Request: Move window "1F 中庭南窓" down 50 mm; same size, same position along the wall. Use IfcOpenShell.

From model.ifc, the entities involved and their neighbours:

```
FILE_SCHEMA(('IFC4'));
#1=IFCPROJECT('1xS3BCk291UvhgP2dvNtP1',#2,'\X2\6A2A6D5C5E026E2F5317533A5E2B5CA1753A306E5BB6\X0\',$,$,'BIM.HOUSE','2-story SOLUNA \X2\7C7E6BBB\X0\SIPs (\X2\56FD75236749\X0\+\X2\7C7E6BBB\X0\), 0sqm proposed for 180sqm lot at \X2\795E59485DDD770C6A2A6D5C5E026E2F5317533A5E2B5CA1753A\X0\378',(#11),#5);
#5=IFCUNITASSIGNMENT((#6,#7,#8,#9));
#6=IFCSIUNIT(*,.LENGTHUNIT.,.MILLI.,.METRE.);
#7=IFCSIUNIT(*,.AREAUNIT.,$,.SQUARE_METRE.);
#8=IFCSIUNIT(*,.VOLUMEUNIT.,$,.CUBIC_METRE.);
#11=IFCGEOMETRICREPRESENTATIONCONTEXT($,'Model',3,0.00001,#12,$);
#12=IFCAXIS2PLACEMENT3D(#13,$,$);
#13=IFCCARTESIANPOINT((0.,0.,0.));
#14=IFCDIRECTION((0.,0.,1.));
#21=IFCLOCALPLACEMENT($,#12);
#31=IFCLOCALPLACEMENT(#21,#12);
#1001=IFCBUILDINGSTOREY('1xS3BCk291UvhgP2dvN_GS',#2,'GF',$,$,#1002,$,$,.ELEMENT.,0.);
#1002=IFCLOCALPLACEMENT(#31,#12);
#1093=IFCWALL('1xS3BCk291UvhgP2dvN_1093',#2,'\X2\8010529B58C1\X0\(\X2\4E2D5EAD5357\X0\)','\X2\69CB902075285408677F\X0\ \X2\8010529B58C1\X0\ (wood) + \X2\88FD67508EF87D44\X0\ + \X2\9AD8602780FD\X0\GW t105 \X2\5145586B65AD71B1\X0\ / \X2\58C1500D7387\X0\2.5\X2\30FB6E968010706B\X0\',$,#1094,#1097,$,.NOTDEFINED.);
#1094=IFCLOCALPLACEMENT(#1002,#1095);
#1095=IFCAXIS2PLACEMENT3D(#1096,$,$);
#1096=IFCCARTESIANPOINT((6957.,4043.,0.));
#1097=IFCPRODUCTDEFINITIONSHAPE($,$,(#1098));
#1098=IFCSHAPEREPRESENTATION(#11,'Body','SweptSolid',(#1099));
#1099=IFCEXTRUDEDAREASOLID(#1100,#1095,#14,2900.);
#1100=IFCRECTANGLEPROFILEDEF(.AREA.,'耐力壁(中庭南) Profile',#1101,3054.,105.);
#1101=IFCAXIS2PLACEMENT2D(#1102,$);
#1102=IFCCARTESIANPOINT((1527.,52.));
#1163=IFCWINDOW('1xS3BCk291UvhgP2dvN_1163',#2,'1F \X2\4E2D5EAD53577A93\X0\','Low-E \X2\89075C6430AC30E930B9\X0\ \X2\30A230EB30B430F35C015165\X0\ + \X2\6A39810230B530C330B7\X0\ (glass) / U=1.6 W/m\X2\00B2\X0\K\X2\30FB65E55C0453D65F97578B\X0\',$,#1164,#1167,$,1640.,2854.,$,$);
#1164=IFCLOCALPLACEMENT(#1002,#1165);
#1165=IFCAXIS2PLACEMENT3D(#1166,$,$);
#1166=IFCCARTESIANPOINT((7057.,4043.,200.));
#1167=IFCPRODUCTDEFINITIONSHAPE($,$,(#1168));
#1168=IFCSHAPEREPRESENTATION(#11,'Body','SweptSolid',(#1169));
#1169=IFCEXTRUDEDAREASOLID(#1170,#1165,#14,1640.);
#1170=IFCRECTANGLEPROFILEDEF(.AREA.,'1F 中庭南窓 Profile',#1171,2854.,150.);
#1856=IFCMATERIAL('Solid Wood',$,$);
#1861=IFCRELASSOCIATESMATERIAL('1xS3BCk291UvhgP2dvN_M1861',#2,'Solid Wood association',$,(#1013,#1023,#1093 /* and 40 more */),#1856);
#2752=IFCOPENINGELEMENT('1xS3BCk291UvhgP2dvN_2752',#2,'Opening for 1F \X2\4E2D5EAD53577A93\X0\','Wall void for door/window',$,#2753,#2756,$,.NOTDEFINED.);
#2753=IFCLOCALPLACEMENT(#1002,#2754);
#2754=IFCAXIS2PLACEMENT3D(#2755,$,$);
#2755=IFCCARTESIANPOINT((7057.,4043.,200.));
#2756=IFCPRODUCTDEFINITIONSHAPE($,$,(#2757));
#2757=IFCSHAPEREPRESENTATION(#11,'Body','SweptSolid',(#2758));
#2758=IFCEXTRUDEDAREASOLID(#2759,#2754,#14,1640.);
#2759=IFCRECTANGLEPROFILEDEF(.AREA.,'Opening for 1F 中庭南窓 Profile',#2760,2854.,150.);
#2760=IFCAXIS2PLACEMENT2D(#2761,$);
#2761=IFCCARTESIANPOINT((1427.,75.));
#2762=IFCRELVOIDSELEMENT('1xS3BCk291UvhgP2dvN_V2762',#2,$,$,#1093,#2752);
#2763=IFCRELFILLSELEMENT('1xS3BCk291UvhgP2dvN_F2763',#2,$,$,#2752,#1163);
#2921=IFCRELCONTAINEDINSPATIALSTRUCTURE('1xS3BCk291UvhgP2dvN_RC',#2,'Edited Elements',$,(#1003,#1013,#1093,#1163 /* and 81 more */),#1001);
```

```python
import numpy as np
import ifcopenshell
import ifcopenshell.api.geometry
import ifcopenshell.util.placement
import ifcopenshell.util.unit

model = ifcopenshell.open("model.ifc")
unit_scale = ifcopenshell.util.unit.calculate_unit_scale(model)

window = model.by_guid("1xS3BCk291UvhgP2dvN_1163")
opening = window.FillsVoids[0].RelatingOpeningElement
dz = -0.05 / unit_scale

shift = np.array([0.0, 0.0, dz])
# The window is not placed relative to its opening, so move both.
for product in (opening, window):
    matrix = ifcopenshell.util.placement.get_local_placement(product.ObjectPlacement)
    matrix[:3, 3] += shift
    ifcopenshell.api.geometry.edit_object_placement(model, product=product, matrix=matrix, is_si=False)

print(f"moved by {dz * unit_scale:+.3f} m")

model.write("model_rev.ifc")
```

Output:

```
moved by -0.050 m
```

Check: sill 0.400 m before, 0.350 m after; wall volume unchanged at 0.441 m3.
